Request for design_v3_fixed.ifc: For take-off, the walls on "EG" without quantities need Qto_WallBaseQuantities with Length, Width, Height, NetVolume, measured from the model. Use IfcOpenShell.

First a look at what the model holds.

```python
import ifcopenshell
import ifcopenshell.util.element
import ifcopenshell.util.unit

model = ifcopenshell.open("design_v3_fixed.ifc")
print(model.schema)
for unit_type in ("LENGTHUNIT", "AREAUNIT", "VOLUMEUNIT"):
    print(unit_type, ifcopenshell.util.unit.calculate_unit_scale(model, unit_type))
storey = next(s for s in model.by_type("IfcBuildingStorey") if s.Name == "EG")
walls = [e for e in ifcopenshell.util.element.get_decomposition(storey) if e.is_a("IfcWall")]
for e in sorted(walls, key=lambda e: e.id()):
    print(e.id(), e.is_a(), e.Name, list(ifcopenshell.util.element.get_psets(e, qtos_only=True)), sep=" | ")
```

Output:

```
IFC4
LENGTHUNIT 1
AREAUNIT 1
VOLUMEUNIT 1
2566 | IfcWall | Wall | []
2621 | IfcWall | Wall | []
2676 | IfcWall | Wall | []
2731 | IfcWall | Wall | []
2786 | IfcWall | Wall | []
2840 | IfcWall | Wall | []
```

```python
import ifcopenshell
import ifcopenshell.api.pset
import ifcopenshell.geom
import ifcopenshell.util.element
import ifcopenshell.util.shape
import ifcopenshell.util.unit

model = ifcopenshell.open("design_v3_fixed.ifc")
unit_scale = ifcopenshell.util.unit.calculate_unit_scale(model)
volume_scale = ifcopenshell.util.unit.calculate_unit_scale(model, "VOLUMEUNIT")
settings = ifcopenshell.geom.settings()

storey = next(s for s in model.by_type("IfcBuildingStorey") if s.Name == "EG")
walls = [e for e in ifcopenshell.util.element.get_decomposition(storey) if e.is_a("IfcWall")]

for e in sorted(walls, key=lambda e: e.id()):
    if ifcopenshell.util.element.get_psets(e, qtos_only=True, should_inherit=False):
        continue
    # Geometry comes back in metres, in the element's own axes.
    shape = ifcopenshell.geom.create_shape(settings, e)
    values = {
        "Length": ifcopenshell.util.shape.get_x(shape.geometry) / unit_scale,
        "Width": ifcopenshell.util.shape.get_y(shape.geometry) / unit_scale,
        "Height": ifcopenshell.util.shape.get_z(shape.geometry) / unit_scale,
        "NetVolume": ifcopenshell.util.shape.get_volume(shape.geometry) / volume_scale,
    }
    qto = ifcopenshell.api.pset.add_qto(model, product=e, name="Qto_WallBaseQuantities")
    ifcopenshell.api.pset.edit_qto(model, qto=qto, properties=values)
    print(e.id(), {k: round(v, 3) for k, v in values.items()})

model.write("design_v3_fixed-out.ifc")
```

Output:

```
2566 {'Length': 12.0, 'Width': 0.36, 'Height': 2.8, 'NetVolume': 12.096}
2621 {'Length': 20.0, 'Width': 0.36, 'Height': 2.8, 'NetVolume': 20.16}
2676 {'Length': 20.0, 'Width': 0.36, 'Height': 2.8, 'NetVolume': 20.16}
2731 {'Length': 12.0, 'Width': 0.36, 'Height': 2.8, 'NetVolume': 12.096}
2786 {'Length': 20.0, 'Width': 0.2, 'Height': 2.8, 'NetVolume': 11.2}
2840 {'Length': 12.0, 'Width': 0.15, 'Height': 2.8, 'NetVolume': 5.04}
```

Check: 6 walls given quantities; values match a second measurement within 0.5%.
